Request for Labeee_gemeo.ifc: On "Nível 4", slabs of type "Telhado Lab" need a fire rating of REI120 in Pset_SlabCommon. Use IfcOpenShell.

First a look at what the model holds.

```python
import ifcopenshell
import ifcopenshell.util.element

model = ifcopenshell.open("Labeee_gemeo.ifc")
print(model.schema)
storey = next(s for s in model.by_type("IfcBuildingStorey") if s.Name == "Nível 4")
slabs = [e for e in ifcopenshell.util.element.get_decomposition(storey) if e.is_a("IfcSlab")]
seen = {}
for e in slabs:
    element_type = ifcopenshell.util.element.get_type(e)
    key = (element_type.Name if element_type != e and element_type else None, ifcopenshell.util.element.get_pset(e, "Pset_SlabCommon", "FireRating"))
    seen[key] = seen.get(key, 0) + 1
for (name, value), count in sorted(seen.items(), key=str):
    print(count, "x", name, "|", value)
```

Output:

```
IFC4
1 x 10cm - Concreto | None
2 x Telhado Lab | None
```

```python
import ifcopenshell
import ifcopenshell.api.pset
import ifcopenshell.util.element

model = ifcopenshell.open("Labeee_gemeo.ifc")

storey = next(s for s in model.by_type("IfcBuildingStorey") if s.Name == "Nível 4")
slabs = [e for e in ifcopenshell.util.element.get_decomposition(storey) if e.is_a("IfcSlab")]

count = 0
for e in slabs:
    element_type = ifcopenshell.util.element.get_type(e)
    if element_type in (None, e) or element_type.Name != "Telhado Lab":
        continue
    # add_pset returns the element's existing set when there is one.
    pset = ifcopenshell.api.pset.add_pset(model, product=e, name="Pset_SlabCommon")
    ifcopenshell.api.pset.edit_pset(model, pset=pset, properties={"FireRating": "REI120"})
    count += 1

print(count, "slabs updated")

model.write("Labeee_gemeo_rev.ifc")
```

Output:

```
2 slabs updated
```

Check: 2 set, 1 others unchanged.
